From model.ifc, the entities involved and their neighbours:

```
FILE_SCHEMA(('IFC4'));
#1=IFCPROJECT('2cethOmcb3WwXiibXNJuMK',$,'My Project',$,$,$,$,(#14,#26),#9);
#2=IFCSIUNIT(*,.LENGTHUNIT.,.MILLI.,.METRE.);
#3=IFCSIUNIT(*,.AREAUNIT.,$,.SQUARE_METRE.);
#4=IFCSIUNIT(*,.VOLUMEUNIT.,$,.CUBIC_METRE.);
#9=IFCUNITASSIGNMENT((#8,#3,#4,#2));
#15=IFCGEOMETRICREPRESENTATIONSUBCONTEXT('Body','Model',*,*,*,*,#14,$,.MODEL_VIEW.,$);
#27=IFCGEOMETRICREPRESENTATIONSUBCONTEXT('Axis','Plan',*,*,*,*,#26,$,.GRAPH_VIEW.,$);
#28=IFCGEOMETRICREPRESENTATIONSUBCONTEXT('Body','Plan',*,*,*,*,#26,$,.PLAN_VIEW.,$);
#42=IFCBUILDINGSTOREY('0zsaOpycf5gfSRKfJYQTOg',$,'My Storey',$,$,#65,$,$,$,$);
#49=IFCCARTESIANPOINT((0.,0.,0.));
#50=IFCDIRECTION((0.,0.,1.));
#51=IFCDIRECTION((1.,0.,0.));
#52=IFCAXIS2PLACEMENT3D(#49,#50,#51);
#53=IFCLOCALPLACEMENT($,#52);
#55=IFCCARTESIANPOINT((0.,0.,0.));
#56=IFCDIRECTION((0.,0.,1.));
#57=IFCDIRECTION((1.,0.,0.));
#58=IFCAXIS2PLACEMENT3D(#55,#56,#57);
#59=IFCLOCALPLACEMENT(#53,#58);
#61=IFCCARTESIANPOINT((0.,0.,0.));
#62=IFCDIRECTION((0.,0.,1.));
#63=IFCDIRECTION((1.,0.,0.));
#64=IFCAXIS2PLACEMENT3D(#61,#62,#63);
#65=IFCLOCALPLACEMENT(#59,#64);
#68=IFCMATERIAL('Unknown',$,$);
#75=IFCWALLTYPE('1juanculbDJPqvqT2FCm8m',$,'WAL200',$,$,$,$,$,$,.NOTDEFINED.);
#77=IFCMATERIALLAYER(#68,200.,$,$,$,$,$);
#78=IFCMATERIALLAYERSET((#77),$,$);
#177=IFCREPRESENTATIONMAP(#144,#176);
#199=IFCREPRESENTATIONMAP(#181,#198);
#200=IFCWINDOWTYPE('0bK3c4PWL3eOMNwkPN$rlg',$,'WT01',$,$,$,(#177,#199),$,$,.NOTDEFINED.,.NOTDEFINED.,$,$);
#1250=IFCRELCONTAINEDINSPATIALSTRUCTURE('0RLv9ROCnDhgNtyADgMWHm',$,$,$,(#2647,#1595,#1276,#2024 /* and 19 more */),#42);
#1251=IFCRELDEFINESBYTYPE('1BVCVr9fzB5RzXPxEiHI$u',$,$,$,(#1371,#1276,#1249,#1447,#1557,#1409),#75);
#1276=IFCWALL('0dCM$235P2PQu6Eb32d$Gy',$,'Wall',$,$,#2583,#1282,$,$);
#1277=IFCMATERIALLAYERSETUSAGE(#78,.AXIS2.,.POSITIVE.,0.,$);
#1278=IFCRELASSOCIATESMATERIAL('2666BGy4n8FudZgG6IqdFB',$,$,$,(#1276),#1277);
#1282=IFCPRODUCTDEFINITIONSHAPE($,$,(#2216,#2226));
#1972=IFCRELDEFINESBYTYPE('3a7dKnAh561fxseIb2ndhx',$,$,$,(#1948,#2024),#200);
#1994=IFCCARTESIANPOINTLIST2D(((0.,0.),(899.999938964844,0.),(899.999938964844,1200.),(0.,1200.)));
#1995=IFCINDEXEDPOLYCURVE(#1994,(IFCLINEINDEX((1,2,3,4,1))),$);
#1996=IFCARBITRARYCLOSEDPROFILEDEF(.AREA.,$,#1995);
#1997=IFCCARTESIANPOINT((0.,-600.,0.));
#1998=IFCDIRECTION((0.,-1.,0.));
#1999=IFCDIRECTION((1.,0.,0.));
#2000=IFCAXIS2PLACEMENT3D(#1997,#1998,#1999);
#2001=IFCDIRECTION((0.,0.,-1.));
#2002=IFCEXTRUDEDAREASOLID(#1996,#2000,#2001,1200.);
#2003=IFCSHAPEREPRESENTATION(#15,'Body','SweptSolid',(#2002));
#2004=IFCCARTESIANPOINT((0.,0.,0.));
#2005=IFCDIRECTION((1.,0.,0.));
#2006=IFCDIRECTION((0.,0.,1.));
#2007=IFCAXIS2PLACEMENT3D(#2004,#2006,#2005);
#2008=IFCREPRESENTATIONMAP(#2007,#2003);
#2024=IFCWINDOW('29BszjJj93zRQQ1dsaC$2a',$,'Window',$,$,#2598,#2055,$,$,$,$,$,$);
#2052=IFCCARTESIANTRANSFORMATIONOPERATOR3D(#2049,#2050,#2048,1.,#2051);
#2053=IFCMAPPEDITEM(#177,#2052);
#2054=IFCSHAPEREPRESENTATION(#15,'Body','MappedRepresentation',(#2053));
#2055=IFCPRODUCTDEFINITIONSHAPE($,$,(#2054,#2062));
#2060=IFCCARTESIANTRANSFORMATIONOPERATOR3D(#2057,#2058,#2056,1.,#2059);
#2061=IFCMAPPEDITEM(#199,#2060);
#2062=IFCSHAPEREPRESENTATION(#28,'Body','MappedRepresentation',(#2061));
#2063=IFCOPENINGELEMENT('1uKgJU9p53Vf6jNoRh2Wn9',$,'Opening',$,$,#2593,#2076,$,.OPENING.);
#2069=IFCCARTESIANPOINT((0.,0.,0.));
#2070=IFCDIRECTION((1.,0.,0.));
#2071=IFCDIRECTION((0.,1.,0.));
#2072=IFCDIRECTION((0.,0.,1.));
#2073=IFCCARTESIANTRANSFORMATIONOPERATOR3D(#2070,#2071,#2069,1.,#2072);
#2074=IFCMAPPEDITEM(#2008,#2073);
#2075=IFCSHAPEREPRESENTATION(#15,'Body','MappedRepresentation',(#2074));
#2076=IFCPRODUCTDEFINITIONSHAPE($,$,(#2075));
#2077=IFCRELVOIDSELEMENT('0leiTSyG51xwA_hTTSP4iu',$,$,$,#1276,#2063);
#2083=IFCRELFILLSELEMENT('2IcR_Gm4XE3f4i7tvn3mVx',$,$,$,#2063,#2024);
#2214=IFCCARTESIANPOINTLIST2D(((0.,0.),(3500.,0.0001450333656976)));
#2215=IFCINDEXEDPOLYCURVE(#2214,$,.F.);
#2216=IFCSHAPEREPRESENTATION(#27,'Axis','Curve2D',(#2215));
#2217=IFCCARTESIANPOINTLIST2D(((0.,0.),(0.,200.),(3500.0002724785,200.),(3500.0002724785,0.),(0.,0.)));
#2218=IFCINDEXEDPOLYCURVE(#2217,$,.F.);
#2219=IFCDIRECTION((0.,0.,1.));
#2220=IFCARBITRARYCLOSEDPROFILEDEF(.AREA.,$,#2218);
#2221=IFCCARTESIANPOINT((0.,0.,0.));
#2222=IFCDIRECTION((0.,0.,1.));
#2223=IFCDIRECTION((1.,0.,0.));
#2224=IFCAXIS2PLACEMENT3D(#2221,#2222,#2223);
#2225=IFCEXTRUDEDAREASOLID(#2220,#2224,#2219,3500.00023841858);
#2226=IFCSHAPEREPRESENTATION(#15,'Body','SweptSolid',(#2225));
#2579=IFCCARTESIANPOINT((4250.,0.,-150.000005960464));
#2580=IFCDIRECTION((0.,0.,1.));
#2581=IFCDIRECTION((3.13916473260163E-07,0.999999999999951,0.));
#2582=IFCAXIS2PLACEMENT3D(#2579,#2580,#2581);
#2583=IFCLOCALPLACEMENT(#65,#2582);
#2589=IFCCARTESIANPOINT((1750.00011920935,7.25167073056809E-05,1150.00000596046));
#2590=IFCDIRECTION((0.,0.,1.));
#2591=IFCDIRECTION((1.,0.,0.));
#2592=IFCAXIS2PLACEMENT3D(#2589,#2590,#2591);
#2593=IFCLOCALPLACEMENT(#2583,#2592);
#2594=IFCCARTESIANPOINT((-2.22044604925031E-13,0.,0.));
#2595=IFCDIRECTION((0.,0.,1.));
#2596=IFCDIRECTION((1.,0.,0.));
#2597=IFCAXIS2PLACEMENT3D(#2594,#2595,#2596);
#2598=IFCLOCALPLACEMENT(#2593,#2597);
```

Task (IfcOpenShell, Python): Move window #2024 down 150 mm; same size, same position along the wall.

```python
import numpy as np
import ifcopenshell
import ifcopenshell.api.geometry
import ifcopenshell.util.placement
import ifcopenshell.util.unit

model = ifcopenshell.open("model.ifc")
unit_scale = ifcopenshell.util.unit.calculate_unit_scale(model)

window = model.by_guid("29BszjJj93zRQQ1dsaC$2a")
opening = window.FillsVoids[0].RelatingOpeningElement
dz = -0.15 / unit_scale

shift = np.array([0.0, 0.0, dz])
# The window is placed relative to its opening, so it follows when the opening moves.
matrix = ifcopenshell.util.placement.get_local_placement(opening.ObjectPlacement)
matrix[:3, 3] += shift
ifcopenshell.api.geometry.edit_object_placement(
    model, product=opening, matrix=matrix, is_si=False, should_transform_children=True
)

print(f"moved by {dz * unit_scale:+.3f} m")

model.write("model_edited.ifc")
```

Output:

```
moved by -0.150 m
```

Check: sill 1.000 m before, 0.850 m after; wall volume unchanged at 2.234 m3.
